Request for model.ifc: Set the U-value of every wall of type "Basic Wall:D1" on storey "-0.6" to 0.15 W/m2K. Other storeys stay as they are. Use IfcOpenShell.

First a look at what the model holds.

```python
import ifcopenshell
import ifcopenshell.util.element

model = ifcopenshell.open("model.ifc")
print(model.schema)
storey = next(s for s in model.by_type("IfcBuildingStorey") if s.Name == "-0.6")
walls = [e for e in ifcopenshell.util.element.get_decomposition(storey) if e.is_a("IfcWall")]
seen = {}
for e in walls:
    element_type = ifcopenshell.util.element.get_type(e)
    key = (element_type.Name if element_type != e and element_type else None, ifcopenshell.util.element.get_pset(e, "Pset_WallCommon", "ThermalTransmittance"))
    seen[key] = seen.get(key, 0) + 1
for (name, value), count in sorted(seen.items(), key=str):
    print(count, "x", name, "|", value)
```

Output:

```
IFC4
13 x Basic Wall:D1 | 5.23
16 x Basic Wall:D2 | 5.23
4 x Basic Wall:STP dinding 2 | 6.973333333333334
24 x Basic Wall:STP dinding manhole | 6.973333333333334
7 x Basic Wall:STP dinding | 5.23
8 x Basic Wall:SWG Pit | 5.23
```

```python
import ifcopenshell
import ifcopenshell.api.pset
import ifcopenshell.util.element

model = ifcopenshell.open("model.ifc")

storey = next(s for s in model.by_type("IfcBuildingStorey") if s.Name == "-0.6")
walls = [e for e in ifcopenshell.util.element.get_decomposition(storey) if e.is_a("IfcWall")]

count = 0
for e in walls:
    element_type = ifcopenshell.util.element.get_type(e)
    if element_type in (None, e) or element_type.Name != "Basic Wall:D1":
        continue
    # add_pset returns the element's existing set when there is one.
    pset = ifcopenshell.api.pset.add_pset(model, product=e, name="Pset_WallCommon")
    ifcopenshell.api.pset.edit_pset(model, pset=pset, properties={"ThermalTransmittance": 0.15})
    count += 1

print(count, "walls updated")

model.write("model_rev.ifc")
```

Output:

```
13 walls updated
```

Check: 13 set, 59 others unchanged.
